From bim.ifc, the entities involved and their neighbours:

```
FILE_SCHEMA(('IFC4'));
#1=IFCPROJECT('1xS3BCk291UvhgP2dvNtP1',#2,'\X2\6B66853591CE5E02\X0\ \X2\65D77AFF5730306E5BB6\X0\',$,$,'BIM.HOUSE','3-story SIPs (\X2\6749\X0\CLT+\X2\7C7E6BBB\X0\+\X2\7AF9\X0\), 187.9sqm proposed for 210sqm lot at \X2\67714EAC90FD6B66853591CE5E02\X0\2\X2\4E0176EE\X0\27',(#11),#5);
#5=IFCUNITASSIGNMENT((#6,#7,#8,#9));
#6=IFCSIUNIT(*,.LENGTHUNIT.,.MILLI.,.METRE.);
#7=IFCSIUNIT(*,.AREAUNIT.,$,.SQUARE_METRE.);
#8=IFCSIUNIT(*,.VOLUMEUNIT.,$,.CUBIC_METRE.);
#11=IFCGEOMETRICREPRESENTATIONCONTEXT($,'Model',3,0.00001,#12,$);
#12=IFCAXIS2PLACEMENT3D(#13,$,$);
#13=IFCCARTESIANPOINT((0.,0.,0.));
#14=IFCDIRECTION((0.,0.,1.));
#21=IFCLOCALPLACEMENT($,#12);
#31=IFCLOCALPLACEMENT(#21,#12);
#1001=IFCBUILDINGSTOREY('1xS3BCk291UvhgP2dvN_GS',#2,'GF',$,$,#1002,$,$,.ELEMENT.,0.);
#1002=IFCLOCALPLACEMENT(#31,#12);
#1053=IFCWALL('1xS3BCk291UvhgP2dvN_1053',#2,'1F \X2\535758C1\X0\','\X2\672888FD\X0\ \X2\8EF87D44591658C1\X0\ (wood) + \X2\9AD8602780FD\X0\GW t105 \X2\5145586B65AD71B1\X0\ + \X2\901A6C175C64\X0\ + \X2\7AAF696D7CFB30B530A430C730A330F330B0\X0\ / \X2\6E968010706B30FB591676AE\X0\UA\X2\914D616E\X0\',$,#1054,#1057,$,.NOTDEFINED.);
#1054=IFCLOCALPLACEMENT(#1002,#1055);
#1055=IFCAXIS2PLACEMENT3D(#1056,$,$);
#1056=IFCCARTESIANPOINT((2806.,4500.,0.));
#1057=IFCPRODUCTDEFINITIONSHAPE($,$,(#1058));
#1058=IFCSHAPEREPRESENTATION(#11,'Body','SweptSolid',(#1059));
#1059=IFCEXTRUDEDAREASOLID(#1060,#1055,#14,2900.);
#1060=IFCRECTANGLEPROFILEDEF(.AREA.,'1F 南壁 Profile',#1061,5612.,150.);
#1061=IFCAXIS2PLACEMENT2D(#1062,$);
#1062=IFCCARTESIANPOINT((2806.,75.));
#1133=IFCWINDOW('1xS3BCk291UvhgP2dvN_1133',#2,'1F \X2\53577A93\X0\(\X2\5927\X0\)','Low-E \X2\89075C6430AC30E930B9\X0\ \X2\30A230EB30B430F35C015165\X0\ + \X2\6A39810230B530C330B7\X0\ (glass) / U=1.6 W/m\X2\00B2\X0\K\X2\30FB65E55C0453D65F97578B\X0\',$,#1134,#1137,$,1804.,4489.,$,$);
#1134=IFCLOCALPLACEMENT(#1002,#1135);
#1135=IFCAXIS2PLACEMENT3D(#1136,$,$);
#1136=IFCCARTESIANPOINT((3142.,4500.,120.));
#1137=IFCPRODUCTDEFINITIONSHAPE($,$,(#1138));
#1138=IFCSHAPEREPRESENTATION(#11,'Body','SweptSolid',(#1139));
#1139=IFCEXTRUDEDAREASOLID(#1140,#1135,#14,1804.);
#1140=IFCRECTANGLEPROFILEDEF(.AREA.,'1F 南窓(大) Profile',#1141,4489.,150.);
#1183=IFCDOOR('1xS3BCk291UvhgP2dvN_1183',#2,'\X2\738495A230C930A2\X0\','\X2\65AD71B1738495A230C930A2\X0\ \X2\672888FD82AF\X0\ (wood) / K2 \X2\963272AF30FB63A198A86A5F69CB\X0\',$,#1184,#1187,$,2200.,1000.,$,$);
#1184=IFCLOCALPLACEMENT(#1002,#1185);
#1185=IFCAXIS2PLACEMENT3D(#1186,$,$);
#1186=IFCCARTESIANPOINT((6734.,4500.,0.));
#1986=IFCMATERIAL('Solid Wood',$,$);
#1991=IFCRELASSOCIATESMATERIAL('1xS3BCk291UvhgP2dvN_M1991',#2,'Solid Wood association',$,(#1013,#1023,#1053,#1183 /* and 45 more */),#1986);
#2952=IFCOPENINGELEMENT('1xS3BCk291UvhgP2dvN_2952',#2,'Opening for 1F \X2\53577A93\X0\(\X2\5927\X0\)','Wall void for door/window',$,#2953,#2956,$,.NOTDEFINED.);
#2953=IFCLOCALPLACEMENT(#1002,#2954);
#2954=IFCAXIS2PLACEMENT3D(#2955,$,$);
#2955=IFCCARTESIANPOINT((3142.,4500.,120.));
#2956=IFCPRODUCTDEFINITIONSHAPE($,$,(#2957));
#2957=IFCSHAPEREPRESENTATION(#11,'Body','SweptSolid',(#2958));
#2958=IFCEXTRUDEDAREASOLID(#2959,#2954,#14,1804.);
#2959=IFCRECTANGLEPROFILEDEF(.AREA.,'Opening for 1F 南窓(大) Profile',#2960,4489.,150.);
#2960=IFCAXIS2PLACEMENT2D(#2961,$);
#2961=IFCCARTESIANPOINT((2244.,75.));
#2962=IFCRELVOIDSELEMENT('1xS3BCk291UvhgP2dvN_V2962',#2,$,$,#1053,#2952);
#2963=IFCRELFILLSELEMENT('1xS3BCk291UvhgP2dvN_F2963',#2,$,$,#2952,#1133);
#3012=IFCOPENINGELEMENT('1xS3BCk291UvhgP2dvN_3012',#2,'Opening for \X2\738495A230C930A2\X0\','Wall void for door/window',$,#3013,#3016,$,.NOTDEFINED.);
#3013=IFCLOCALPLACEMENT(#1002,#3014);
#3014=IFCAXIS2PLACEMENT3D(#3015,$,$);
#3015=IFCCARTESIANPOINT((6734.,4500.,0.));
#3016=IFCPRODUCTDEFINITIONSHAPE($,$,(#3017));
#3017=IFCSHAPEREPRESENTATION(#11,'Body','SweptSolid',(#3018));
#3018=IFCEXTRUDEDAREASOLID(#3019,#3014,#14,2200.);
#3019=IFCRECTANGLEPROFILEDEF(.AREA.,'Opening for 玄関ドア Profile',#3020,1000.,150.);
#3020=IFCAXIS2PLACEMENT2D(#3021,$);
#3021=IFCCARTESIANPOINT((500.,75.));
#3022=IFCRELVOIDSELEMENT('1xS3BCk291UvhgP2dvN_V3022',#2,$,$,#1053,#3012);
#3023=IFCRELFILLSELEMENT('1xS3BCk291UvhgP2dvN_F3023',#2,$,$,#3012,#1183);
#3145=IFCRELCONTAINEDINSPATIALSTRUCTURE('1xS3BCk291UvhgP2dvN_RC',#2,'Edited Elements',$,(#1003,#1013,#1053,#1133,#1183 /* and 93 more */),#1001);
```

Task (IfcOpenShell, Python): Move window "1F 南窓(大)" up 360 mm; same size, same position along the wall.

```python
import numpy as np
import ifcopenshell
import ifcopenshell.api.geometry
import ifcopenshell.util.placement
import ifcopenshell.util.unit

model = ifcopenshell.open("bim.ifc")
unit_scale = ifcopenshell.util.unit.calculate_unit_scale(model)

window = model.by_guid("1xS3BCk291UvhgP2dvN_1133")
opening = window.FillsVoids[0].RelatingOpeningElement
dz = 0.36 / unit_scale

shift = np.array([0.0, 0.0, dz])
# The window is not placed relative to its opening, so move both.
for product in (opening, window):
    matrix = ifcopenshell.util.placement.get_local_placement(product.ObjectPlacement)
    matrix[:3, 3] += shift
    ifcopenshell.api.geometry.edit_object_placement(model, product=product, matrix=matrix, is_si=False)

print(f"moved by {dz * unit_scale:+.3f} m")

model.write("bim_edited.ifc")
```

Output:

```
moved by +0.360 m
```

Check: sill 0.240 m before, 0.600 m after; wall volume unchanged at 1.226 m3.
